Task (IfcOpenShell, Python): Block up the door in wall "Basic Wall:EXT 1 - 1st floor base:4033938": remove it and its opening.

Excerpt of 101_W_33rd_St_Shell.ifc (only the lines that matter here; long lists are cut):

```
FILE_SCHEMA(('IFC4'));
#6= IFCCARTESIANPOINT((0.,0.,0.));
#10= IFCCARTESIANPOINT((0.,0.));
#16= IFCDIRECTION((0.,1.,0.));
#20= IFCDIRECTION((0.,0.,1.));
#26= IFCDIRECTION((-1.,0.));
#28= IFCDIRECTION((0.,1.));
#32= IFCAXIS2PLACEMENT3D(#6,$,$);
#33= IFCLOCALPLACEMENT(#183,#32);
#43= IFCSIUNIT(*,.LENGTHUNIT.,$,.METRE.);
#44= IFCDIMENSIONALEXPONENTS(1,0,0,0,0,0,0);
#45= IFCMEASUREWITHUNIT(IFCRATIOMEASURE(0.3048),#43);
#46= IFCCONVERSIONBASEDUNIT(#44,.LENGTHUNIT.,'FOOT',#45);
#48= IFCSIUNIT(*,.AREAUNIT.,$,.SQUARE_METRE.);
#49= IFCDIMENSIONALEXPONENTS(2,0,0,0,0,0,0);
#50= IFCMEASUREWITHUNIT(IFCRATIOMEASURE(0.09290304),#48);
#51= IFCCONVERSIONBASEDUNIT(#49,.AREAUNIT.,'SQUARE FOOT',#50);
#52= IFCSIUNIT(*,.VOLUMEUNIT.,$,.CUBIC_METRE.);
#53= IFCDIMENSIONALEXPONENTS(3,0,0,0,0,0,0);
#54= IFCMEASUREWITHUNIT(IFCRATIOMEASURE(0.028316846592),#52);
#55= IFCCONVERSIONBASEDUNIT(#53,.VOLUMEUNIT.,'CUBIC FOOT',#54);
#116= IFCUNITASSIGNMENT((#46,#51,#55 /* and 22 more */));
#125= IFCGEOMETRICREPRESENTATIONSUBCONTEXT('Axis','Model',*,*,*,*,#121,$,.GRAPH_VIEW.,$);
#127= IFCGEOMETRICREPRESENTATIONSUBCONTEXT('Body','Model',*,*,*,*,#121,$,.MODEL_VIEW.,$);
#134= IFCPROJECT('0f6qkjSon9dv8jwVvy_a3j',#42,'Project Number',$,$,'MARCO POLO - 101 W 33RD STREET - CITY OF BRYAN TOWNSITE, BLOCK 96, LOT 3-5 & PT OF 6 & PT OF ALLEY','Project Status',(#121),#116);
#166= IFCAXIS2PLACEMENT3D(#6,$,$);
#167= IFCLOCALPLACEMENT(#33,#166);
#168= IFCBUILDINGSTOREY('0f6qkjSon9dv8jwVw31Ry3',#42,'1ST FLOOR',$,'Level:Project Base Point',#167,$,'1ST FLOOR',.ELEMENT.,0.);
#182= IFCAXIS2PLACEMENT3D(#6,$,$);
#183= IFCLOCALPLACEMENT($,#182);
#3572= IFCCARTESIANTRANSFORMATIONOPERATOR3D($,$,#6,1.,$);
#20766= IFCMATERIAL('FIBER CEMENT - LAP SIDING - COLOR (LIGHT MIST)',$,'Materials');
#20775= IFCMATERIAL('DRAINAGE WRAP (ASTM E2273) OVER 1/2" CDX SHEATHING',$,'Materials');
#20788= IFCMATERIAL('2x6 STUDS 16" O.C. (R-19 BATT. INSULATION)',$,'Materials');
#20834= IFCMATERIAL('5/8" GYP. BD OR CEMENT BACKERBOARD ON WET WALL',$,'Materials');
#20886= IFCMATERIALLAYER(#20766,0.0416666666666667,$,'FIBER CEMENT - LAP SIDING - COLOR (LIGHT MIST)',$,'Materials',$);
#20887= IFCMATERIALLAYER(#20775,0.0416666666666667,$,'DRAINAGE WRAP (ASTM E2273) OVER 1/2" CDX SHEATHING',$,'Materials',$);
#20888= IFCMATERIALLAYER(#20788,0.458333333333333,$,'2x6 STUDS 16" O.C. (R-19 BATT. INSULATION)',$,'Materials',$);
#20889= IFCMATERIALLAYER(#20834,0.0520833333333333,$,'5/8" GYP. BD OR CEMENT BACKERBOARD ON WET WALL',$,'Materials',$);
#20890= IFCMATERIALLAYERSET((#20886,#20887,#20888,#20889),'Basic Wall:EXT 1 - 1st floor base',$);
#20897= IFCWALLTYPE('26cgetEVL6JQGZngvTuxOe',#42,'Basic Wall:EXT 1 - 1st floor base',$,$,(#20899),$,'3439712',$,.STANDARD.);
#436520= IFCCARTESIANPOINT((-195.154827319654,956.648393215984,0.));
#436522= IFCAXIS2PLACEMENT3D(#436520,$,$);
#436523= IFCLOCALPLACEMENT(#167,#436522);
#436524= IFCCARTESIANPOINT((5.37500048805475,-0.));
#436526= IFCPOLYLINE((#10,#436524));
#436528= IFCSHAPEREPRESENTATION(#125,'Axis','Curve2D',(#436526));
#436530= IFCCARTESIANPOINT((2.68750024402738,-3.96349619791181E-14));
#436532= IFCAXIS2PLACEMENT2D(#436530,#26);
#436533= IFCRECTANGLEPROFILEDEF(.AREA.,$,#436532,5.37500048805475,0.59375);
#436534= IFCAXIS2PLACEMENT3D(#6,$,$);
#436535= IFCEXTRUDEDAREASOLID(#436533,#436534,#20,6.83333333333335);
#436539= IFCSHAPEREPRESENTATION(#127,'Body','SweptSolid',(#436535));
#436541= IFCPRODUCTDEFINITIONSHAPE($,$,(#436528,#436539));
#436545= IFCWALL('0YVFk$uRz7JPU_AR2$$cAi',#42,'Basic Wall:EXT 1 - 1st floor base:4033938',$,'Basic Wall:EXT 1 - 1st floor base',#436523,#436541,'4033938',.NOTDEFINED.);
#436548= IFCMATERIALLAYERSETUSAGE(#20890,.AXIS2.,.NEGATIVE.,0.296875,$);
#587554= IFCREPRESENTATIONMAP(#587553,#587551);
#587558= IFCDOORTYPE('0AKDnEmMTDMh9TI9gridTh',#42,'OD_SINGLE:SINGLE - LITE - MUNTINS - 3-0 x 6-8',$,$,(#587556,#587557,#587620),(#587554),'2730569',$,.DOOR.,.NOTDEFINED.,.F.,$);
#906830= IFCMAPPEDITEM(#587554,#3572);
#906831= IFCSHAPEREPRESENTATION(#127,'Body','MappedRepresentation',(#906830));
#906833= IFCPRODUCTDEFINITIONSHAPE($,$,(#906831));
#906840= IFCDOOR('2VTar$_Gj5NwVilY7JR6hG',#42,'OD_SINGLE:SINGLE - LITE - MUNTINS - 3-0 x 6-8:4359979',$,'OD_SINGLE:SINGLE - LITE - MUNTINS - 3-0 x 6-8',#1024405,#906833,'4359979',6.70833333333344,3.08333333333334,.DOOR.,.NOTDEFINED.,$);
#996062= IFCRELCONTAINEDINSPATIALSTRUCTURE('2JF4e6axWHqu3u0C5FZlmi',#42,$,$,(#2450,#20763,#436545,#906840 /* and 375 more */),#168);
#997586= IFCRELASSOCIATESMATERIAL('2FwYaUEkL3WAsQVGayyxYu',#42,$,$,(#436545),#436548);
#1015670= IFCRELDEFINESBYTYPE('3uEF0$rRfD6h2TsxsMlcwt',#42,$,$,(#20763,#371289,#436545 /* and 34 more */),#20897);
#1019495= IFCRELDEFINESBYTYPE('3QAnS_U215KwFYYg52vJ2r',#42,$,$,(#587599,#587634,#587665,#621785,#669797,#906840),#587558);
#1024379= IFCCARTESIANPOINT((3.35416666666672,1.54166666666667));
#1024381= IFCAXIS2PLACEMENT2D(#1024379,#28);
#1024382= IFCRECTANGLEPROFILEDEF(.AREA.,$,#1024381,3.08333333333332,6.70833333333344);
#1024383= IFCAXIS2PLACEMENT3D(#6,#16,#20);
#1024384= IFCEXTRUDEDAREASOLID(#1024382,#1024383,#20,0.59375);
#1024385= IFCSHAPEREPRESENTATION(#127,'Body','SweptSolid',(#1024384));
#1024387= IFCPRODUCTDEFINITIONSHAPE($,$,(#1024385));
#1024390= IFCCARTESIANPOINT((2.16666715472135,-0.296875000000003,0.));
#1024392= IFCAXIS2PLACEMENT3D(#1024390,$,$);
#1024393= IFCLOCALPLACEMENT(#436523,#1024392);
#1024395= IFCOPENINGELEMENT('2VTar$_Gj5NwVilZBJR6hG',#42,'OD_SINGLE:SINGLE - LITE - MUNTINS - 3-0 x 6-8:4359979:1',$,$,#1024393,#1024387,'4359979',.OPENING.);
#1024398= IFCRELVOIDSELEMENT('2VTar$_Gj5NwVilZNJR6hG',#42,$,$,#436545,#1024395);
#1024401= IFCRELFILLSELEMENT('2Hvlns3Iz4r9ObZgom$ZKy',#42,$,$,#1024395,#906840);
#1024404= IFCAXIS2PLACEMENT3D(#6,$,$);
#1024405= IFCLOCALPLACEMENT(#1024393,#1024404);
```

```python
import ifcopenshell
import ifcopenshell.api.feature
import ifcopenshell.api.root
import ifcopenshell.geom
import ifcopenshell.util.shape

model = ifcopenshell.open("101_W_33rd_St_Shell.ifc")
settings = ifcopenshell.geom.settings()


def volume(element):
    """Net volume in cubic metres, openings subtracted."""
    shape = ifcopenshell.geom.create_shape(settings, element)
    return ifcopenshell.util.shape.get_volume(shape.geometry)


door = model.by_guid("2VTar$_Gj5NwVilY7JR6hG")
opening = door.FillsVoids[0].RelatingOpeningElement
wall = opening.VoidsElements[0].RelatingBuildingElement
before = volume(wall)

ifcopenshell.api.root.remove_product(model, product=door)
ifcopenshell.api.feature.remove_feature(model, feature=opening)

after = volume(wall)

print(f"wall volume {before:.3f} -> {after:.3f} m3")

model.write("101_W_33rd_St_Shell_updated.ifc")
```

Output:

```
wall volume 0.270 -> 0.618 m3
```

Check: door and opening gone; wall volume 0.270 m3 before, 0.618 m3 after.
